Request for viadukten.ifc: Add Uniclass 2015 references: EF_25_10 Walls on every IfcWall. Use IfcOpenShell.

First a look at what the model holds.

```python
import ifcopenshell

model = ifcopenshell.open("viadukten.ifc")
print(model.schema)
print("classifications:", [c.Name for c in model.by_type("IfcClassification")])
for ifc_class in ("IfcDoor", "IfcRoof", "IfcStair", "IfcWall", "IfcWindow"):
    print(ifc_class, len(model.by_type(ifc_class)))
```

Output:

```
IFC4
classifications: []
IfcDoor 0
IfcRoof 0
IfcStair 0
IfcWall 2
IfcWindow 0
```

```python
import ifcopenshell
import ifcopenshell.api.classification

model = ifcopenshell.open("viadukten.ifc")

system = ifcopenshell.api.classification.add_classification(model, classification="Uniclass 2015")

codes = {
    "IfcWall": ("EF_25_10", "Walls"),
}
for ifc_class, (code, name) in codes.items():
    products = model.by_type(ifc_class)
    ifcopenshell.api.classification.add_reference(
        model, products=products, classification=system, identification=code, name=name
    )
    print(code, len(products))

model.write("viadukten_updated.ifc")
```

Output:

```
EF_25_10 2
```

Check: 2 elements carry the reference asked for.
